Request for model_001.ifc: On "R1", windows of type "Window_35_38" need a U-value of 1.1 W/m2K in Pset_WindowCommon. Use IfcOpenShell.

First a look at what the model holds.

```python
import ifcopenshell
import ifcopenshell.util.element

model = ifcopenshell.open("model_001.ifc")
print(model.schema)
storey = next(s for s in model.by_type("IfcBuildingStorey") if s.Name == "R1")
windows = [e for e in ifcopenshell.util.element.get_decomposition(storey) if e.is_a("IfcWindow")]
seen = {}
for e in windows:
    element_type = ifcopenshell.util.element.get_type(e)
    key = (element_type.Name if element_type != e and element_type else None, ifcopenshell.util.element.get_pset(e, "Pset_WindowCommon", "ThermalTransmittance"))
    seen[key] = seen.get(key, 0) + 1
for (name, value), count in sorted(seen.items(), key=str):
    print(count, "x", name, "|", value)
```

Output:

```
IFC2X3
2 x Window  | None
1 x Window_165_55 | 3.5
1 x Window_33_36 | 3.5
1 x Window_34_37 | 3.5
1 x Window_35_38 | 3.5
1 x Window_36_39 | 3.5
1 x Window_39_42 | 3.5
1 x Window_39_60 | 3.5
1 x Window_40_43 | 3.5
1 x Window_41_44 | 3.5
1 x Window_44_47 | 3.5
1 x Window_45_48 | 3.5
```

```python
import ifcopenshell
import ifcopenshell.api.pset
import ifcopenshell.util.element

model = ifcopenshell.open("model_001.ifc")

storey = next(s for s in model.by_type("IfcBuildingStorey") if s.Name == "R1")
windows = [e for e in ifcopenshell.util.element.get_decomposition(storey) if e.is_a("IfcWindow")]

count = 0
for e in windows:
    element_type = ifcopenshell.util.element.get_type(e)
    if element_type in (None, e) or element_type.Name != "Window_35_38":
        continue
    # add_pset returns the element's existing set when there is one.
    pset = ifcopenshell.api.pset.add_pset(model, product=e, name="Pset_WindowCommon")
    ifcopenshell.api.pset.edit_pset(model, pset=pset, properties={"ThermalTransmittance": 1.1})
    count += 1

print(count, "windows updated")

model.write("model_001_rev.ifc")
```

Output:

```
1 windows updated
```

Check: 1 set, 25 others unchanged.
